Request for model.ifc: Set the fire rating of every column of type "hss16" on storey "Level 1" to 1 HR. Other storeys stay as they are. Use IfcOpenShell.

First a look at what the model holds.

```python
import ifcopenshell
import ifcopenshell.util.element

model = ifcopenshell.open("model.ifc")
print(model.schema)
storey = next(s for s in model.by_type("IfcBuildingStorey") if s.Name == "Level 1")
columns = [e for e in ifcopenshell.util.element.get_decomposition(storey) if e.is_a("IfcColumn")]
seen = {}
for e in columns:
    element_type = ifcopenshell.util.element.get_type(e)
    key = (element_type.Name if element_type != e and element_type else None, ifcopenshell.util.element.get_pset(e, "Pset_ColumnCommon", "FireRating"))
    seen[key] = seen.get(key, 0) + 1
for (name, value), count in sorted(seen.items(), key=str):
    print(count, "x", name, "|", value)
```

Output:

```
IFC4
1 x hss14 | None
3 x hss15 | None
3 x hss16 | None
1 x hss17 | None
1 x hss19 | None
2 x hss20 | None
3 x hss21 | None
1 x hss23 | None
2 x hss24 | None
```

```python
import ifcopenshell
import ifcopenshell.api.pset
import ifcopenshell.util.element

model = ifcopenshell.open("model.ifc")

storey = next(s for s in model.by_type("IfcBuildingStorey") if s.Name == "Level 1")
columns = [e for e in ifcopenshell.util.element.get_decomposition(storey) if e.is_a("IfcColumn")]

count = 0
for e in columns:
    element_type = ifcopenshell.util.element.get_type(e)
    if element_type in (None, e) or element_type.Name != "hss16":
        continue
    # add_pset returns the element's existing set when there is one.
    pset = ifcopenshell.api.pset.add_pset(model, product=e, name="Pset_ColumnCommon")
    ifcopenshell.api.pset.edit_pset(model, pset=pset, properties={"FireRating": "1 HR"})
    count += 1

print(count, "columns updated")

model.write("model_edited.ifc")
```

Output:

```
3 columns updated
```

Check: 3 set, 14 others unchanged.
